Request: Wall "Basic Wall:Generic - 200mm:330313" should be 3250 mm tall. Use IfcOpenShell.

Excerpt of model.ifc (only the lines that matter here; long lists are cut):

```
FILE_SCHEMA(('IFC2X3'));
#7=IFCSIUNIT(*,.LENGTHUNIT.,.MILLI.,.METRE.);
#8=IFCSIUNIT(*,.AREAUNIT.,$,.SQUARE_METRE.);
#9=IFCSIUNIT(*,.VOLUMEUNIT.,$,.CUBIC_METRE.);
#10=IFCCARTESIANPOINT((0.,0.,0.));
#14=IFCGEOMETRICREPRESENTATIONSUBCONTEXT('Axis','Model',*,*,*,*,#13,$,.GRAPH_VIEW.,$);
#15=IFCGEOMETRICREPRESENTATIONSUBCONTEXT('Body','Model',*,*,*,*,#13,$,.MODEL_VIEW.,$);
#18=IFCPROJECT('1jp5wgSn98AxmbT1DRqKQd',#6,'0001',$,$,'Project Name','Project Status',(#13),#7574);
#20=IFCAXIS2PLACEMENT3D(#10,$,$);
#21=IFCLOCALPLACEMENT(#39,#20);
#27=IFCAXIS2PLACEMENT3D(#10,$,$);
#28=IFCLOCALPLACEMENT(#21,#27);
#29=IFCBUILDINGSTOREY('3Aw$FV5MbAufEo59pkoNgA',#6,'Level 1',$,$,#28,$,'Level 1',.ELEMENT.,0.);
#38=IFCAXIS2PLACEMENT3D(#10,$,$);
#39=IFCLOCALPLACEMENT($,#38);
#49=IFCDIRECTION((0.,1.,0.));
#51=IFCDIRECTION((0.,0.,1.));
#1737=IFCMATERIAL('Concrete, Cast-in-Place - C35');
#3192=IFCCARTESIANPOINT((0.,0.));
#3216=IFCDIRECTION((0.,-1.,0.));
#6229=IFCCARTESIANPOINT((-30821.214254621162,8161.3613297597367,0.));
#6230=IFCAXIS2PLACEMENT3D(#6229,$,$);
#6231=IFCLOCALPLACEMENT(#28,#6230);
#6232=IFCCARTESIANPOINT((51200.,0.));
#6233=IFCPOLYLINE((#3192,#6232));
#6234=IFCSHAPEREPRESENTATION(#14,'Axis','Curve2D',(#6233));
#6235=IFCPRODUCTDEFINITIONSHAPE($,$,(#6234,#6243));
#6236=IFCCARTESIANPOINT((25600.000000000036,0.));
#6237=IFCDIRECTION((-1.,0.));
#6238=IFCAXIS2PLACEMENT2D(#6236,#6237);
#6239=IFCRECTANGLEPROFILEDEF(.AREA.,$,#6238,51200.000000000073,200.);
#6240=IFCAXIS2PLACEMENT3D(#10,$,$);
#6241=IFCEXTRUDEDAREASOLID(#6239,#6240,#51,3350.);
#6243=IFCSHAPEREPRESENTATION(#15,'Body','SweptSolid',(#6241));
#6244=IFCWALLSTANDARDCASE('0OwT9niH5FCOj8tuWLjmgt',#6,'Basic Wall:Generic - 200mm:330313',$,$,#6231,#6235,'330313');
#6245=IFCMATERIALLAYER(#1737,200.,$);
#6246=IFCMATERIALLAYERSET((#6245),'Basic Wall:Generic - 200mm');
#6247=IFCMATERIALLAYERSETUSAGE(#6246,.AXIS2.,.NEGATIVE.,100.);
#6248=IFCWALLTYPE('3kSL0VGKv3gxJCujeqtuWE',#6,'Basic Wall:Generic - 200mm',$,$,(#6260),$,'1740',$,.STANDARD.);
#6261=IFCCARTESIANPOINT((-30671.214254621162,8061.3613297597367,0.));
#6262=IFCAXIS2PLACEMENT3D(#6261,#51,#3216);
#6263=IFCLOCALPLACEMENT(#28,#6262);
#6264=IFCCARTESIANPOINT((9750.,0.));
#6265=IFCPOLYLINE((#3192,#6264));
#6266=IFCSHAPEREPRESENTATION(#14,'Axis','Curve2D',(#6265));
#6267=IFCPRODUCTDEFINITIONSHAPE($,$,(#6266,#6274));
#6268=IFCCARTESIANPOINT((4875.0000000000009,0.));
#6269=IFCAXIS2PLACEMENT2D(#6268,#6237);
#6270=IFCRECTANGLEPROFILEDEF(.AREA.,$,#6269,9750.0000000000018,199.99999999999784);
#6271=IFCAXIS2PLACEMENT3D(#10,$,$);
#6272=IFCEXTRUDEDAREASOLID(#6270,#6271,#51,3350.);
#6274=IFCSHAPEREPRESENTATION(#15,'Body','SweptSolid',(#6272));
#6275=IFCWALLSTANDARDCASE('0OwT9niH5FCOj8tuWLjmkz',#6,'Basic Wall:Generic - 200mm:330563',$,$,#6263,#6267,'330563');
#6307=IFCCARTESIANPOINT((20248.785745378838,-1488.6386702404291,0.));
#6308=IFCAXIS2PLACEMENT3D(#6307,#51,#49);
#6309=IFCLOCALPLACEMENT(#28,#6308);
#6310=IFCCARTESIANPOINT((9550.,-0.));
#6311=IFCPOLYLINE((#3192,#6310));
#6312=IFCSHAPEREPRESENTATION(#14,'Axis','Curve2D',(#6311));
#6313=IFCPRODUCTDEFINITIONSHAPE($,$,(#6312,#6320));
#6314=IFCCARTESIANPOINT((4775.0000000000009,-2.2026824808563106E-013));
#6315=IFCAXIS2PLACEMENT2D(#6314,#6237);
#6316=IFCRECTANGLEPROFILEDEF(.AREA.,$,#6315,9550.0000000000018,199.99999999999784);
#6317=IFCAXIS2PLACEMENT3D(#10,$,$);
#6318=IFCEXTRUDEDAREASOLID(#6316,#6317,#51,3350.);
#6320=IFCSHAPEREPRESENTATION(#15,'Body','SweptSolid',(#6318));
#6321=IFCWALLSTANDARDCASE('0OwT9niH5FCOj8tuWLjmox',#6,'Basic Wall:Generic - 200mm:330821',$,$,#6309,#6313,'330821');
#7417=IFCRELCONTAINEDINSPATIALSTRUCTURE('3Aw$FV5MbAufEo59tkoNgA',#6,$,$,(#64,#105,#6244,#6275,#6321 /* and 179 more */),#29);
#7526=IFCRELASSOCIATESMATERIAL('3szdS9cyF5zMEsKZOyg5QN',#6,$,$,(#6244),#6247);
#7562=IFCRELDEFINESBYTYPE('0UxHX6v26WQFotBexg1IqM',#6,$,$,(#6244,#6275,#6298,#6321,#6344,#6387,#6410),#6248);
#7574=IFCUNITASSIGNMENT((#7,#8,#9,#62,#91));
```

```python
import ifcopenshell
import ifcopenshell.geom
import ifcopenshell.util.representation
import ifcopenshell.util.shape
import ifcopenshell.util.unit

model = ifcopenshell.open("model.ifc")
unit_scale = ifcopenshell.util.unit.calculate_unit_scale(model)
settings = ifcopenshell.geom.settings()


def volume(element):
    """Net volume in cubic metres, openings subtracted."""
    shape = ifcopenshell.geom.create_shape(settings, element)
    return ifcopenshell.util.shape.get_volume(shape.geometry)


wall = model.by_id(6244)
before = volume(wall)

body = ifcopenshell.util.representation.get_representation(wall, "Model", "Body")
solid = body.Items[0]
old_height = solid.Depth
solid.Depth = 3.25 / unit_scale
after = volume(wall)

print(f"height {old_height:g} -> {solid.Depth:g}, volume {before:.3f} -> {after:.3f} m3")

model.write("model_rev.ifc")
```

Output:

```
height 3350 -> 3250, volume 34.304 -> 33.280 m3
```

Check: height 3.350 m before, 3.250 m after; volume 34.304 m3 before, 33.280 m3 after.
